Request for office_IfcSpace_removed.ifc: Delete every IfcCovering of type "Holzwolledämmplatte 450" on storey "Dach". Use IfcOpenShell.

First a look at what the model holds.

```python
import ifcopenshell
import ifcopenshell.util.element

model = ifcopenshell.open("office_IfcSpace_removed.ifc")
print(model.schema)
storey = next(s for s in model.by_type("IfcBuildingStorey") if s.Name == "Dach")
coverings = [e for e in ifcopenshell.util.element.get_decomposition(storey) if e.is_a("IfcCovering")]
seen = {}
for e in coverings:
    element_type = ifcopenshell.util.element.get_type(e)
    name = element_type.Name if element_type not in (None, e) else None
    seen[name] = seen.get(name, 0) + 1
for name, count in sorted(seen.items(), key=str):
    print(count, "x", name)
```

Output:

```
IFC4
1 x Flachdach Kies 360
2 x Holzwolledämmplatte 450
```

```python
import ifcopenshell
import ifcopenshell.api.root
import ifcopenshell.util.element

model = ifcopenshell.open("office_IfcSpace_removed.ifc")

storey = next(s for s in model.by_type("IfcBuildingStorey") if s.Name == "Dach")
coverings = [e for e in ifcopenshell.util.element.get_decomposition(storey) if e.is_a("IfcCovering")]
targets = [e for e in coverings if (t := ifcopenshell.util.element.get_type(e)) not in (None, e) and t.Name == "Holzwolledämmplatte 450"]

for e in targets:
    ifcopenshell.api.root.remove_product(model, product=e)
print(len(targets), "removed")

model.write("office_IfcSpace_removed-out.ifc")
```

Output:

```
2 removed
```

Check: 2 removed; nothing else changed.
